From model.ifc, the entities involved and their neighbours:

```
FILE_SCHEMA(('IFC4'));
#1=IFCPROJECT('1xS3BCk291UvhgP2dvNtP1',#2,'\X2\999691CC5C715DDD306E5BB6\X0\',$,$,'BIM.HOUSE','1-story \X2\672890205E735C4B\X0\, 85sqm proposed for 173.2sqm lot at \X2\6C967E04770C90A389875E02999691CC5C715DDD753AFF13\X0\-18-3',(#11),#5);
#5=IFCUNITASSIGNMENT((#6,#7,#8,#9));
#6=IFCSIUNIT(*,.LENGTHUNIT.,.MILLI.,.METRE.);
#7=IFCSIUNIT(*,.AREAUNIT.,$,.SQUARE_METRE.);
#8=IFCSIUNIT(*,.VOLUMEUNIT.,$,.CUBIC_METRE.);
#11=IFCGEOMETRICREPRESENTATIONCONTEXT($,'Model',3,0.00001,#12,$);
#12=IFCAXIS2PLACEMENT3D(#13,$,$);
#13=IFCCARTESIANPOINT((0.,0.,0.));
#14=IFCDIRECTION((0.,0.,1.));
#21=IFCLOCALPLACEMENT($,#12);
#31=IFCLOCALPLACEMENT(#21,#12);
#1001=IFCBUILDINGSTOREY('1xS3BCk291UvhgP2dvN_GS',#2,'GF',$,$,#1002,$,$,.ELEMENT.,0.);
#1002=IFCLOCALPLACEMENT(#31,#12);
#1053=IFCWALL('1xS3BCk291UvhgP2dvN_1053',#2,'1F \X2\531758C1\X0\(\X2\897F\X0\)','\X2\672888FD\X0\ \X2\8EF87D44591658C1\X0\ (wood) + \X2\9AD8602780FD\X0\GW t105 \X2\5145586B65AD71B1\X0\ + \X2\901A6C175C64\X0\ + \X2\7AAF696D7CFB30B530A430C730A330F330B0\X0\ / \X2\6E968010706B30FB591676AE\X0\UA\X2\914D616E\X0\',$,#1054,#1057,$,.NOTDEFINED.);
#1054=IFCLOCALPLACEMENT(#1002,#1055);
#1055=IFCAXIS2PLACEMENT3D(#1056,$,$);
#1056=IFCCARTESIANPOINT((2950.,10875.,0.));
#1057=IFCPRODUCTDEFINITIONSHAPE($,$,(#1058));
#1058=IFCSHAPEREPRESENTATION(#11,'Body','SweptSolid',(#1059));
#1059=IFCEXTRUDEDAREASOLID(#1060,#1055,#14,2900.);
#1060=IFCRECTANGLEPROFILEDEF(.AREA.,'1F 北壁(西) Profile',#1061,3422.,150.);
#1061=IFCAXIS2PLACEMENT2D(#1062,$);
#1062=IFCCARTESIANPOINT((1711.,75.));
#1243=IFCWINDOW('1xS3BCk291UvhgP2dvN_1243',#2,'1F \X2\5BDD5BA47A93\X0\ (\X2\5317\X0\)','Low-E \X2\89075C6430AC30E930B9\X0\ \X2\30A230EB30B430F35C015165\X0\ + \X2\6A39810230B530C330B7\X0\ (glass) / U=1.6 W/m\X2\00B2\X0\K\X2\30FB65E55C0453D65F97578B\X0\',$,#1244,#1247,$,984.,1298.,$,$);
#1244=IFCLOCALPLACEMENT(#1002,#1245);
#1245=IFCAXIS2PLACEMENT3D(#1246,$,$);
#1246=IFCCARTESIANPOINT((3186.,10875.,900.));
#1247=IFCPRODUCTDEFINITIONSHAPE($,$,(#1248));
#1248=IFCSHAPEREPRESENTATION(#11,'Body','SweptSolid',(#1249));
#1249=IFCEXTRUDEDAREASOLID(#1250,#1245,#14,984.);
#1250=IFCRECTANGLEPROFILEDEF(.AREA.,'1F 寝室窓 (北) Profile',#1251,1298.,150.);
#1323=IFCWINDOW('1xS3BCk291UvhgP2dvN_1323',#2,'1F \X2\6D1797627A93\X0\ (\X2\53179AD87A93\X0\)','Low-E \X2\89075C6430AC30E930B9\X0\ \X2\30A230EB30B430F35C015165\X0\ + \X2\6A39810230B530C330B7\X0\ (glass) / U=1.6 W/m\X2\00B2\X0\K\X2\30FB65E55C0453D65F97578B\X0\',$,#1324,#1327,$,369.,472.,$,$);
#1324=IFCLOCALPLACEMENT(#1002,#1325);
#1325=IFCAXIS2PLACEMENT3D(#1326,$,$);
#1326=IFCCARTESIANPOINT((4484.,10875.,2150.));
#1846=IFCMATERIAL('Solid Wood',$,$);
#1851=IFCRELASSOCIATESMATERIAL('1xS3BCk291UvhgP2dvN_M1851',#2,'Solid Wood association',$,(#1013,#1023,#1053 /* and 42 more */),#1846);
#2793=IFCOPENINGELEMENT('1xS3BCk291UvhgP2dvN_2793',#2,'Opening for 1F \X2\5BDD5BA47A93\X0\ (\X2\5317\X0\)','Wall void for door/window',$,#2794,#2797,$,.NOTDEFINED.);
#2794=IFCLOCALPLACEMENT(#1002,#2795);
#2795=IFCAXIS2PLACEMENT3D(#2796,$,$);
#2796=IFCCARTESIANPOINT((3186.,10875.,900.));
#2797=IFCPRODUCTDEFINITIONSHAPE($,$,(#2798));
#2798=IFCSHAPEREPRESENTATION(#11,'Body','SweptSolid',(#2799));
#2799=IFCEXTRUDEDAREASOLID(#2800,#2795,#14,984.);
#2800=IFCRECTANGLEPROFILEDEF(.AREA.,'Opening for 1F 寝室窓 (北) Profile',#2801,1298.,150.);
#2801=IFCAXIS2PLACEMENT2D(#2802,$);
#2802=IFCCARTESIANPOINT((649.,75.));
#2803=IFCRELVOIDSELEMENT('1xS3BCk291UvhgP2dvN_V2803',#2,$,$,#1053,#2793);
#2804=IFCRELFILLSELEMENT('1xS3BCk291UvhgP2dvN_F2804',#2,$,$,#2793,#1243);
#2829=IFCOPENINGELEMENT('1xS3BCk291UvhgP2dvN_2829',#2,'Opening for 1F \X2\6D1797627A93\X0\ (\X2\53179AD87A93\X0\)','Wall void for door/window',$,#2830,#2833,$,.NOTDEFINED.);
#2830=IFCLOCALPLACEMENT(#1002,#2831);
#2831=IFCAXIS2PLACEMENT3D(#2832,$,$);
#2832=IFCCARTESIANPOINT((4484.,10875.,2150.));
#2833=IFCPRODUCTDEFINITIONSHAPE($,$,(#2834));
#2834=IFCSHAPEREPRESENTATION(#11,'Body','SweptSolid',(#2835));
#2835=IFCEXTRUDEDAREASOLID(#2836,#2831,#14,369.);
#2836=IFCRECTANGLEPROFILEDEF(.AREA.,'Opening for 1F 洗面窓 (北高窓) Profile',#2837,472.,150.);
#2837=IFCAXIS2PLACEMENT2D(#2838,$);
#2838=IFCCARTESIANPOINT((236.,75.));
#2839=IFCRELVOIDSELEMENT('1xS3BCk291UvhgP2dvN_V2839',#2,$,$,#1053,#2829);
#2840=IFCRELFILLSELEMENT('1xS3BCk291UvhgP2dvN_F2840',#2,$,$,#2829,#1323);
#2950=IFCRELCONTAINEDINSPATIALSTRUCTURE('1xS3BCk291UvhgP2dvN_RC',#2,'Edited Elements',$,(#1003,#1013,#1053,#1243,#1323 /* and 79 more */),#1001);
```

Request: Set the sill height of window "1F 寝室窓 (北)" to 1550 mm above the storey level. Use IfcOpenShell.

```python
import numpy as np
import ifcopenshell
import ifcopenshell.api.geometry
import ifcopenshell.geom
import ifcopenshell.util.element
import ifcopenshell.util.placement
import ifcopenshell.util.shape
import ifcopenshell.util.unit

model = ifcopenshell.open("model.ifc")
unit_scale = ifcopenshell.util.unit.calculate_unit_scale(model)

window = model.by_guid("1xS3BCk291UvhgP2dvN_1243")
opening = window.FillsVoids[0].RelatingOpeningElement
storey = ifcopenshell.util.element.get_container(window, ifc_class="IfcBuildingStorey")
level = ifcopenshell.util.placement.get_local_placement(storey.ObjectPlacement)[2, 3]

# The opening's origin need not be at the sill, so measure its lowest point.
shape = ifcopenshell.geom.create_shape(ifcopenshell.geom.settings(), opening)
bottom = ifcopenshell.util.shape.get_shape_bottom_elevation(shape, shape.geometry) / unit_scale
dz = level + 1.55 / unit_scale - bottom

shift = np.array([0.0, 0.0, dz])
# The window is not placed relative to its opening, so move both.
for product in (opening, window):
    matrix = ifcopenshell.util.placement.get_local_placement(product.ObjectPlacement)
    matrix[:3, 3] += shift
    ifcopenshell.api.geometry.edit_object_placement(model, product=product, matrix=matrix, is_si=False)

print(f"moved by {dz * unit_scale:+.3f} m")

model.write("model-out.ifc")
```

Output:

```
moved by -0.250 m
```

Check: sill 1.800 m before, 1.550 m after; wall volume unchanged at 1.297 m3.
